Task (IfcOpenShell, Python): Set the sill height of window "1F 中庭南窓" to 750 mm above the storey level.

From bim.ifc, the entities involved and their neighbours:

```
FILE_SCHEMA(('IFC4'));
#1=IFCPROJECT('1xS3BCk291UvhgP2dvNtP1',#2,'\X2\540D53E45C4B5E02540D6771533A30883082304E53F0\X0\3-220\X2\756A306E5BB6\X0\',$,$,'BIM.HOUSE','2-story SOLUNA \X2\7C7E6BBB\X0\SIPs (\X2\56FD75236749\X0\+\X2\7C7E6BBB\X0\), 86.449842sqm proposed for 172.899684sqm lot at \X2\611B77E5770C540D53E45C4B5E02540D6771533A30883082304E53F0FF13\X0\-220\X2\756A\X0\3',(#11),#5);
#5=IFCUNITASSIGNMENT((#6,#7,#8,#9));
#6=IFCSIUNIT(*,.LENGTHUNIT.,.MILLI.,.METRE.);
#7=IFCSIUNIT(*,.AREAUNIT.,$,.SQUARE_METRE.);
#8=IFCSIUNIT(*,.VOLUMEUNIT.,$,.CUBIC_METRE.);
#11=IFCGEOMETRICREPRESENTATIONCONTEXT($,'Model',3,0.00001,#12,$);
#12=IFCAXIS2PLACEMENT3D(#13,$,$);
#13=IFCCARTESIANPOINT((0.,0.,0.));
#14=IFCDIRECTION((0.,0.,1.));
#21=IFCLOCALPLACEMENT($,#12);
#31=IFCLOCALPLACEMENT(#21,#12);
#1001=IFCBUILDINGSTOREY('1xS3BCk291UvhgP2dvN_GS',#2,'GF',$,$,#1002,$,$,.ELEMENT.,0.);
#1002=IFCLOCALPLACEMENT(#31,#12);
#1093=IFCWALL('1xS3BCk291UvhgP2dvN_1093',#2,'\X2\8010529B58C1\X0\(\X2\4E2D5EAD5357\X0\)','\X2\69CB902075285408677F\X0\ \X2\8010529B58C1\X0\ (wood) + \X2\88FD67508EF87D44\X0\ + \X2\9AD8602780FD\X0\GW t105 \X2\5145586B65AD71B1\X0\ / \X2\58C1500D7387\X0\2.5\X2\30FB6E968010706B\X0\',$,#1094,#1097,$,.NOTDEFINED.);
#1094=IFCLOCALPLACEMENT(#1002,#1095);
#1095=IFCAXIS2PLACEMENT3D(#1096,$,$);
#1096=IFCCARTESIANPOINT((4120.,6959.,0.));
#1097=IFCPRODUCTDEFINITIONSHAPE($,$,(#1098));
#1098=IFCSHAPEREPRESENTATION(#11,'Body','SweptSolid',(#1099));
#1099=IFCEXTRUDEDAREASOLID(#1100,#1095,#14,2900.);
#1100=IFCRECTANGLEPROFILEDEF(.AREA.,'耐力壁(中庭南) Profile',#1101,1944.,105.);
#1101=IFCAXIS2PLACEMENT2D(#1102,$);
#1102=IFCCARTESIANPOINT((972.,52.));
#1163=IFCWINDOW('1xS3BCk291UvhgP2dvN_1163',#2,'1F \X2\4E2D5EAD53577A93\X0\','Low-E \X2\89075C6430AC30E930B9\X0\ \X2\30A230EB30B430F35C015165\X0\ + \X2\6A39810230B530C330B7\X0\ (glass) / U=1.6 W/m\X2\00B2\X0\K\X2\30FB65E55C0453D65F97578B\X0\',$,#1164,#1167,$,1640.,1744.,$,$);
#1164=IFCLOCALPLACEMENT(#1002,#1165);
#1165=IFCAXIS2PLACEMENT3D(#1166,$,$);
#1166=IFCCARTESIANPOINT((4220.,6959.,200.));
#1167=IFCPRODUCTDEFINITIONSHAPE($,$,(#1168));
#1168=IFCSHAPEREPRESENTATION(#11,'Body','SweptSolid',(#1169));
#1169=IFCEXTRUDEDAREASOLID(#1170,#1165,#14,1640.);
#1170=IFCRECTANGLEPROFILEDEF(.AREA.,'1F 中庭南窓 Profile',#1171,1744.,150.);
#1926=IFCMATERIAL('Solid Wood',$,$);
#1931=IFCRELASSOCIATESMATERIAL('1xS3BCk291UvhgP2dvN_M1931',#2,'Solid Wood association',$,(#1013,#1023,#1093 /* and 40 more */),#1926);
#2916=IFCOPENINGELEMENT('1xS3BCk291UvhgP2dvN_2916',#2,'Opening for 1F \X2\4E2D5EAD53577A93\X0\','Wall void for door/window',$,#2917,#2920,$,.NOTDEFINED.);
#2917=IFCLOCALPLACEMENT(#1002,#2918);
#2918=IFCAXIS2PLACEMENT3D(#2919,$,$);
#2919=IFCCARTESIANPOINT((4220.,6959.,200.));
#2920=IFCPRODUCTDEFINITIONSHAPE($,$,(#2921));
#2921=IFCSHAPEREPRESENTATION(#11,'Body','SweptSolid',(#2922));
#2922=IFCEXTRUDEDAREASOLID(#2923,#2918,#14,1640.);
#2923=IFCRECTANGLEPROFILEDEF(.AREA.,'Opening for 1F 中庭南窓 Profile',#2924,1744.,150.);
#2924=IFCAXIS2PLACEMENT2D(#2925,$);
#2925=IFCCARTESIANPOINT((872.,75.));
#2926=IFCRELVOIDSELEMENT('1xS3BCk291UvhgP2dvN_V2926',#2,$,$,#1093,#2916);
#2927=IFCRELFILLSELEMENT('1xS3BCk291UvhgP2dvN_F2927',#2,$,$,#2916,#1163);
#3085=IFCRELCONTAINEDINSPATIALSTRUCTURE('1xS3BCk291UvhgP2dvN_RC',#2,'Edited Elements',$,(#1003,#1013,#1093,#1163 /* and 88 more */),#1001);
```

```python
import numpy as np
import ifcopenshell
import ifcopenshell.api.geometry
import ifcopenshell.geom
import ifcopenshell.util.element
import ifcopenshell.util.placement
import ifcopenshell.util.shape
import ifcopenshell.util.unit

model = ifcopenshell.open("bim.ifc")
unit_scale = ifcopenshell.util.unit.calculate_unit_scale(model)

window = model.by_guid("1xS3BCk291UvhgP2dvN_1163")
opening = window.FillsVoids[0].RelatingOpeningElement
storey = ifcopenshell.util.element.get_container(window, ifc_class="IfcBuildingStorey")
level = ifcopenshell.util.placement.get_local_placement(storey.ObjectPlacement)[2, 3]

# The opening's origin need not be at the sill, so measure its lowest point.
shape = ifcopenshell.geom.create_shape(ifcopenshell.geom.settings(), opening)
bottom = ifcopenshell.util.shape.get_shape_bottom_elevation(shape, shape.geometry) / unit_scale
dz = level + 0.75 / unit_scale - bottom

shift = np.array([0.0, 0.0, dz])
# The window is not placed relative to its opening, so move both.
for product in (opening, window):
    matrix = ifcopenshell.util.placement.get_local_placement(product.ObjectPlacement)
    matrix[:3, 3] += shift
    ifcopenshell.api.geometry.edit_object_placement(model, product=product, matrix=matrix, is_si=False)

print(f"moved by {dz * unit_scale:+.3f} m")

model.write("bim_v2.ifc")
```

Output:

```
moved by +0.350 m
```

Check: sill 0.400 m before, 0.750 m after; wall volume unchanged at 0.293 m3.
